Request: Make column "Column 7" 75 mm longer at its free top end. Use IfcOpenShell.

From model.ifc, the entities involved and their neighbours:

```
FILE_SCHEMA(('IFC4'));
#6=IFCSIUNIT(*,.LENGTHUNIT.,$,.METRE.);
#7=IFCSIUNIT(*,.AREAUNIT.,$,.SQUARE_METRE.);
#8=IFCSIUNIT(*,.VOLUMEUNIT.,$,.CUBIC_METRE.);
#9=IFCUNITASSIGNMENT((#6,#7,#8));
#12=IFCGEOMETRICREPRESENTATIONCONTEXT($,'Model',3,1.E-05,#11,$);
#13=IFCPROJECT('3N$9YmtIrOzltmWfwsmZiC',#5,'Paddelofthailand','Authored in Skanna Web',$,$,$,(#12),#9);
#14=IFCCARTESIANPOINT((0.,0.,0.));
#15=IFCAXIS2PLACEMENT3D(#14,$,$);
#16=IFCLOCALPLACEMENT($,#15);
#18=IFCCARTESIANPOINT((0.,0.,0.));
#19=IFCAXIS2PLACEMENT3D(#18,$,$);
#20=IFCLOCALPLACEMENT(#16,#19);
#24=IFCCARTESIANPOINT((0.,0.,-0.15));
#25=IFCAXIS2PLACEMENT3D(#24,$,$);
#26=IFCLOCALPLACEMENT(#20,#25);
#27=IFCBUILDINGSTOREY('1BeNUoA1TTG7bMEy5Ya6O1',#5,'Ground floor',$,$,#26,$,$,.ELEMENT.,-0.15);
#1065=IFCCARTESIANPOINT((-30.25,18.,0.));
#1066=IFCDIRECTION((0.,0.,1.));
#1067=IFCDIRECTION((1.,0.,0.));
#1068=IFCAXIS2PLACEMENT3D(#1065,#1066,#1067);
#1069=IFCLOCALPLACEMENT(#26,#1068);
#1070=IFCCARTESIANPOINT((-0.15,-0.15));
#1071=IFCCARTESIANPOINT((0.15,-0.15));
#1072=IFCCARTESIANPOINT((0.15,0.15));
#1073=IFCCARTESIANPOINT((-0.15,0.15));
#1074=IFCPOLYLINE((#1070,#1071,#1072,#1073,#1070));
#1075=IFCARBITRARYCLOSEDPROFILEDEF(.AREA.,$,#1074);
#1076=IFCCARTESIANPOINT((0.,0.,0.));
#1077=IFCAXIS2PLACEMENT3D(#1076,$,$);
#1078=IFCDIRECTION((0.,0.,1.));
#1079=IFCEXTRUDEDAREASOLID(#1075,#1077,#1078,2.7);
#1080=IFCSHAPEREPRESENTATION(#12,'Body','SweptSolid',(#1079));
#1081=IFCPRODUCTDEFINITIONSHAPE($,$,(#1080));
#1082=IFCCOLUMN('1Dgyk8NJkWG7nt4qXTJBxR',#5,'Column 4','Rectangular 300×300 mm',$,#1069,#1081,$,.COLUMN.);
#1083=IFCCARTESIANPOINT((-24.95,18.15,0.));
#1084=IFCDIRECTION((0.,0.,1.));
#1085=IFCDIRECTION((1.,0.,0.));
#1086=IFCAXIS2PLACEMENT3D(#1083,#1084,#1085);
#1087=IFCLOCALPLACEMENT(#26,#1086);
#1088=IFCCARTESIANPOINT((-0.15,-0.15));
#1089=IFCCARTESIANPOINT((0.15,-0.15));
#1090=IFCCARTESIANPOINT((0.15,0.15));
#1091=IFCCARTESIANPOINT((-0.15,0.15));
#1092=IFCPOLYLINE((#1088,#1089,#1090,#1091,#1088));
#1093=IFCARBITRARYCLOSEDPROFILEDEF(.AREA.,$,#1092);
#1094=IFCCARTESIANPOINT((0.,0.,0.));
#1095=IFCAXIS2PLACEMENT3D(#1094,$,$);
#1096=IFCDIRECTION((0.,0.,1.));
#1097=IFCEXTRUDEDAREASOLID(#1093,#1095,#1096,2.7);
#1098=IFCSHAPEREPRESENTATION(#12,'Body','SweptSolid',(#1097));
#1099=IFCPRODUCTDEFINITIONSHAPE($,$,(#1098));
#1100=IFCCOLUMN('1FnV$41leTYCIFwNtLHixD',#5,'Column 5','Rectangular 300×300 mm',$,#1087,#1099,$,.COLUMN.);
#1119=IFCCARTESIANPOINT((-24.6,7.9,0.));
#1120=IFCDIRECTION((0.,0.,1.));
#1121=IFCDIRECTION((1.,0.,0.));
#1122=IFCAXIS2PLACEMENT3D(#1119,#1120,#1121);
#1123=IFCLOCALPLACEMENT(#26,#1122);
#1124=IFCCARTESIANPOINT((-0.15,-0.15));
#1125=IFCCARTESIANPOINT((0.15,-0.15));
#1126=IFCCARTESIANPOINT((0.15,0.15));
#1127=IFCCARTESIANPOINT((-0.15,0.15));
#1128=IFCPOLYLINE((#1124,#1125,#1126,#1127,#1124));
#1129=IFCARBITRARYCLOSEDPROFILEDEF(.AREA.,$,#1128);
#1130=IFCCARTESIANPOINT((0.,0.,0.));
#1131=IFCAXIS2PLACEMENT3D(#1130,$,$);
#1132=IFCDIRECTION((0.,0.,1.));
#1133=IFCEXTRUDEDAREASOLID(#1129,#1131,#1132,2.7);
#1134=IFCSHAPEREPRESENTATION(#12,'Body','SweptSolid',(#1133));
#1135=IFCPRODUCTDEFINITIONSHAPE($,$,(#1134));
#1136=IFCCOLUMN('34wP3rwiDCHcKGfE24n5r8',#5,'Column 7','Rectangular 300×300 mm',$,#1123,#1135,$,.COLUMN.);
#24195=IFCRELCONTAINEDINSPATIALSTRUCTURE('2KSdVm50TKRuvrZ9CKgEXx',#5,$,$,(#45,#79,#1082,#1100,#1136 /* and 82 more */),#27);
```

```python
import ifcopenshell

model = ifcopenshell.open("model.ifc")

member = model.by_id(1136)
change = 0.075

# The extrusion runs towards the end named, so only its depth changes.
body = next(r for r in member.Representation.Representations if r.RepresentationIdentifier == "Body")
solid = body.Items[0]
old_length = solid.Depth
solid.Depth += change

print(f"length {old_length:g} -> {solid.Depth:g}")

model.write("model_v2.ifc")
```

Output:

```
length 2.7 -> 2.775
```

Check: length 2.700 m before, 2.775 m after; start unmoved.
